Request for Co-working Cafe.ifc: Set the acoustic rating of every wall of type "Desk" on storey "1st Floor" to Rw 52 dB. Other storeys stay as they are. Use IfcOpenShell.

First a look at what the model holds.

```python
import ifcopenshell
import ifcopenshell.util.element

model = ifcopenshell.open("Co-working Cafe.ifc")
print(model.schema)
storey = next(s for s in model.by_type("IfcBuildingStorey") if s.Name == "1st Floor")
walls = [e for e in ifcopenshell.util.element.get_decomposition(storey) if e.is_a("IfcWall")]
seen = {}
for e in walls:
    element_type = ifcopenshell.util.element.get_type(e)
    key = (element_type.Name if element_type != e and element_type else None, ifcopenshell.util.element.get_pset(e, "Pset_WallCommon", "AcousticRating"))
    seen[key] = seen.get(key, 0) + 1
for (name, value), count in sorted(seen.items(), key=str):
    print(count, "x", name, "|", value)
```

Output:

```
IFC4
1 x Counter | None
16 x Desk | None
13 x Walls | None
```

```python
import ifcopenshell
import ifcopenshell.api.pset
import ifcopenshell.util.element

model = ifcopenshell.open("Co-working Cafe.ifc")

storey = next(s for s in model.by_type("IfcBuildingStorey") if s.Name == "1st Floor")
walls = [e for e in ifcopenshell.util.element.get_decomposition(storey) if e.is_a("IfcWall")]

count = 0
for e in walls:
    element_type = ifcopenshell.util.element.get_type(e)
    if element_type in (None, e) or element_type.Name != "Desk":
        continue
    # add_pset returns the element's existing set when there is one.
    pset = ifcopenshell.api.pset.add_pset(model, product=e, name="Pset_WallCommon")
    ifcopenshell.api.pset.edit_pset(model, pset=pset, properties={"AcousticRating": "Rw 52 dB"})
    count += 1

print(count, "walls updated")

model.write("Co-working Cafe-out.ifc")
```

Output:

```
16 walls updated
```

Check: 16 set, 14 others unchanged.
